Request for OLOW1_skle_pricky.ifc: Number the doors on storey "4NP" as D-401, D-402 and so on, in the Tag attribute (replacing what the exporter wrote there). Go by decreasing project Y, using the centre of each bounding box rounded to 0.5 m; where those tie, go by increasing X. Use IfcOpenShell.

First a look at what the model holds.

```python
import ifcopenshell
import ifcopenshell.util.element
import ifcopenshell.util.placement

model = ifcopenshell.open("OLOW1_skle_pricky.ifc")
print(model.schema)
storey = next(s for s in model.by_type("IfcBuildingStorey") if s.Name == "4NP")
doors = [e for e in ifcopenshell.util.element.get_decomposition(storey) if e.is_a("IfcDoor")]
for e in sorted(doors, key=lambda e: e.id()):
    origin = ifcopenshell.util.placement.get_local_placement(e.ObjectPlacement)[:3, 3]
    print(e.id(), e.Tag, e.Name, origin.round(2) + 0.0, sep=" | ")
```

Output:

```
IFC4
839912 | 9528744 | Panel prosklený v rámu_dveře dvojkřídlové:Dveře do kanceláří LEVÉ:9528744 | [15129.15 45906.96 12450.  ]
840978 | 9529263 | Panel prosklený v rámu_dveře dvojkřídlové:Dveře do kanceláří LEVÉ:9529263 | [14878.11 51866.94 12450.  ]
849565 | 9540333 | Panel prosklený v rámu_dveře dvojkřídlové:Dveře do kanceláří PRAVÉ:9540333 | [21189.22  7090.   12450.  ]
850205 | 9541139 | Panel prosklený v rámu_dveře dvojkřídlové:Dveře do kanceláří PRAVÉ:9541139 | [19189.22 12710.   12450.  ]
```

```python
import ifcopenshell
import ifcopenshell.geom
import ifcopenshell.util.element
import ifcopenshell.util.shape

model = ifcopenshell.open("OLOW1_skle_pricky.ifc")
settings = ifcopenshell.geom.settings()
settings.set("use-world-coords", True)


def centre(element):
    shape = ifcopenshell.geom.create_shape(settings, element)
    return ifcopenshell.util.shape.get_bbox_centroid(shape.geometry)


storey = next(s for s in model.by_type("IfcBuildingStorey") if s.Name == "4NP")
doors = [e for e in ifcopenshell.util.element.get_decomposition(storey) if e.is_a("IfcDoor")]

# Insertion points can sit at a corner or the storey origin, so sort by the geometry (in metres).
centres = {e: centre(e) for e in doors}
doors.sort(key=lambda e: (-round(centres[e][1] / 0.5), centres[e][0]))

for i, e in enumerate(doors, start=1):
    number = f"D-4{i:02d}"
    e.Tag = number
    print(e.id(), number)

model.write("OLOW1_skle_pricky_v2.ifc")
```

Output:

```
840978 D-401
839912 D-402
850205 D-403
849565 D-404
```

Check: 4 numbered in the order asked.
